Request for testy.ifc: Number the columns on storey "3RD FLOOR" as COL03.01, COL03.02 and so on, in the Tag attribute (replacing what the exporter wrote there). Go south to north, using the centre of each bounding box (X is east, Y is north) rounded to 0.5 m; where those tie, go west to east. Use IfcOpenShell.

First a look at what the model holds.

```python
import ifcopenshell
import ifcopenshell.util.element
import ifcopenshell.util.placement

model = ifcopenshell.open("testy.ifc")
print(model.schema)
storey = next(s for s in model.by_type("IfcBuildingStorey") if s.Name == "3RD FLOOR")
columns = [e for e in ifcopenshell.util.element.get_decomposition(storey) if e.is_a("IfcColumn")]
for e in sorted(columns, key=lambda e: e.id()):
    origin = ifcopenshell.util.placement.get_local_placement(e.ObjectPlacement)[:3, 3]
    print(e.id(), e.Tag, e.Name, origin.round(2) + 0.0, sep=" | ")
```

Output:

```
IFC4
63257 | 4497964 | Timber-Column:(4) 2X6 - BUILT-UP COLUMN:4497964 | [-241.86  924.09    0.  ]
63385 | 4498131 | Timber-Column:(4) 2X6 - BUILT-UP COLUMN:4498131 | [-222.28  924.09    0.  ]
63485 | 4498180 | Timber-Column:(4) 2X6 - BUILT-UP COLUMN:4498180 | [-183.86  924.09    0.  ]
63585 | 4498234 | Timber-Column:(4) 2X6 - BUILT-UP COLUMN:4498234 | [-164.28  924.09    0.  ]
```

```python
import ifcopenshell
import ifcopenshell.geom
import ifcopenshell.util.element
import ifcopenshell.util.shape

model = ifcopenshell.open("testy.ifc")
settings = ifcopenshell.geom.settings()
settings.set("use-world-coords", True)


def centre(element):
    shape = ifcopenshell.geom.create_shape(settings, element)
    return ifcopenshell.util.shape.get_bbox_centroid(shape.geometry)


storey = next(s for s in model.by_type("IfcBuildingStorey") if s.Name == "3RD FLOOR")
columns = [e for e in ifcopenshell.util.element.get_decomposition(storey) if e.is_a("IfcColumn")]

# Insertion points can sit at a corner or the storey origin, so sort by the geometry (in metres).
centres = {e: centre(e) for e in columns}
columns.sort(key=lambda e: (round(centres[e][1] / 0.5), centres[e][0]))

for i, e in enumerate(columns, start=1):
    number = f"COL03.{i:02d}"
    e.Tag = number
    print(e.id(), number)

model.write("testy_rev.ifc")
```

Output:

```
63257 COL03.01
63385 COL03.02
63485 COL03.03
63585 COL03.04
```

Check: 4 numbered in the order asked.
